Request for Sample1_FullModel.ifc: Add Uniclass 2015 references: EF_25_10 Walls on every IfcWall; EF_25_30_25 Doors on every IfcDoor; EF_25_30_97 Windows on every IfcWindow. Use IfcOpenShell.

First a look at what the model holds.

```python
import ifcopenshell

model = ifcopenshell.open("Sample1_FullModel.ifc")
print(model.schema)
print("classifications:", [c.Name for c in model.by_type("IfcClassification")])
for ifc_class in ("IfcDoor", "IfcRoof", "IfcStair", "IfcWall", "IfcWindow"):
    print(ifc_class, len(model.by_type(ifc_class)))
```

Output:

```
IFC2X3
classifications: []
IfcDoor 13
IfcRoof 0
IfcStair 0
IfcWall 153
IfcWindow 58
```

```python
import ifcopenshell
import ifcopenshell.api.classification

model = ifcopenshell.open("Sample1_FullModel.ifc")

# IFC2X3 requires Source and Edition and has no link from the project to the system.
system = model.create_entity("IfcClassification", Source="NBS", Edition="2015", Name="Uniclass 2015")

codes = {
    "IfcWall": ("EF_25_10", "Walls"),
    "IfcDoor": ("EF_25_30_25", "Doors"),
    "IfcWindow": ("EF_25_30_97", "Windows"),
}
for ifc_class, (code, name) in codes.items():
    products = model.by_type(ifc_class)
    ifcopenshell.api.classification.add_reference(
        model, products=products, classification=system, identification=code, name=name
    )
    print(code, len(products))

model.write("Sample1_FullModel_updated.ifc")
```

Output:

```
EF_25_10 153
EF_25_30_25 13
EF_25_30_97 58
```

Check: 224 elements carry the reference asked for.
